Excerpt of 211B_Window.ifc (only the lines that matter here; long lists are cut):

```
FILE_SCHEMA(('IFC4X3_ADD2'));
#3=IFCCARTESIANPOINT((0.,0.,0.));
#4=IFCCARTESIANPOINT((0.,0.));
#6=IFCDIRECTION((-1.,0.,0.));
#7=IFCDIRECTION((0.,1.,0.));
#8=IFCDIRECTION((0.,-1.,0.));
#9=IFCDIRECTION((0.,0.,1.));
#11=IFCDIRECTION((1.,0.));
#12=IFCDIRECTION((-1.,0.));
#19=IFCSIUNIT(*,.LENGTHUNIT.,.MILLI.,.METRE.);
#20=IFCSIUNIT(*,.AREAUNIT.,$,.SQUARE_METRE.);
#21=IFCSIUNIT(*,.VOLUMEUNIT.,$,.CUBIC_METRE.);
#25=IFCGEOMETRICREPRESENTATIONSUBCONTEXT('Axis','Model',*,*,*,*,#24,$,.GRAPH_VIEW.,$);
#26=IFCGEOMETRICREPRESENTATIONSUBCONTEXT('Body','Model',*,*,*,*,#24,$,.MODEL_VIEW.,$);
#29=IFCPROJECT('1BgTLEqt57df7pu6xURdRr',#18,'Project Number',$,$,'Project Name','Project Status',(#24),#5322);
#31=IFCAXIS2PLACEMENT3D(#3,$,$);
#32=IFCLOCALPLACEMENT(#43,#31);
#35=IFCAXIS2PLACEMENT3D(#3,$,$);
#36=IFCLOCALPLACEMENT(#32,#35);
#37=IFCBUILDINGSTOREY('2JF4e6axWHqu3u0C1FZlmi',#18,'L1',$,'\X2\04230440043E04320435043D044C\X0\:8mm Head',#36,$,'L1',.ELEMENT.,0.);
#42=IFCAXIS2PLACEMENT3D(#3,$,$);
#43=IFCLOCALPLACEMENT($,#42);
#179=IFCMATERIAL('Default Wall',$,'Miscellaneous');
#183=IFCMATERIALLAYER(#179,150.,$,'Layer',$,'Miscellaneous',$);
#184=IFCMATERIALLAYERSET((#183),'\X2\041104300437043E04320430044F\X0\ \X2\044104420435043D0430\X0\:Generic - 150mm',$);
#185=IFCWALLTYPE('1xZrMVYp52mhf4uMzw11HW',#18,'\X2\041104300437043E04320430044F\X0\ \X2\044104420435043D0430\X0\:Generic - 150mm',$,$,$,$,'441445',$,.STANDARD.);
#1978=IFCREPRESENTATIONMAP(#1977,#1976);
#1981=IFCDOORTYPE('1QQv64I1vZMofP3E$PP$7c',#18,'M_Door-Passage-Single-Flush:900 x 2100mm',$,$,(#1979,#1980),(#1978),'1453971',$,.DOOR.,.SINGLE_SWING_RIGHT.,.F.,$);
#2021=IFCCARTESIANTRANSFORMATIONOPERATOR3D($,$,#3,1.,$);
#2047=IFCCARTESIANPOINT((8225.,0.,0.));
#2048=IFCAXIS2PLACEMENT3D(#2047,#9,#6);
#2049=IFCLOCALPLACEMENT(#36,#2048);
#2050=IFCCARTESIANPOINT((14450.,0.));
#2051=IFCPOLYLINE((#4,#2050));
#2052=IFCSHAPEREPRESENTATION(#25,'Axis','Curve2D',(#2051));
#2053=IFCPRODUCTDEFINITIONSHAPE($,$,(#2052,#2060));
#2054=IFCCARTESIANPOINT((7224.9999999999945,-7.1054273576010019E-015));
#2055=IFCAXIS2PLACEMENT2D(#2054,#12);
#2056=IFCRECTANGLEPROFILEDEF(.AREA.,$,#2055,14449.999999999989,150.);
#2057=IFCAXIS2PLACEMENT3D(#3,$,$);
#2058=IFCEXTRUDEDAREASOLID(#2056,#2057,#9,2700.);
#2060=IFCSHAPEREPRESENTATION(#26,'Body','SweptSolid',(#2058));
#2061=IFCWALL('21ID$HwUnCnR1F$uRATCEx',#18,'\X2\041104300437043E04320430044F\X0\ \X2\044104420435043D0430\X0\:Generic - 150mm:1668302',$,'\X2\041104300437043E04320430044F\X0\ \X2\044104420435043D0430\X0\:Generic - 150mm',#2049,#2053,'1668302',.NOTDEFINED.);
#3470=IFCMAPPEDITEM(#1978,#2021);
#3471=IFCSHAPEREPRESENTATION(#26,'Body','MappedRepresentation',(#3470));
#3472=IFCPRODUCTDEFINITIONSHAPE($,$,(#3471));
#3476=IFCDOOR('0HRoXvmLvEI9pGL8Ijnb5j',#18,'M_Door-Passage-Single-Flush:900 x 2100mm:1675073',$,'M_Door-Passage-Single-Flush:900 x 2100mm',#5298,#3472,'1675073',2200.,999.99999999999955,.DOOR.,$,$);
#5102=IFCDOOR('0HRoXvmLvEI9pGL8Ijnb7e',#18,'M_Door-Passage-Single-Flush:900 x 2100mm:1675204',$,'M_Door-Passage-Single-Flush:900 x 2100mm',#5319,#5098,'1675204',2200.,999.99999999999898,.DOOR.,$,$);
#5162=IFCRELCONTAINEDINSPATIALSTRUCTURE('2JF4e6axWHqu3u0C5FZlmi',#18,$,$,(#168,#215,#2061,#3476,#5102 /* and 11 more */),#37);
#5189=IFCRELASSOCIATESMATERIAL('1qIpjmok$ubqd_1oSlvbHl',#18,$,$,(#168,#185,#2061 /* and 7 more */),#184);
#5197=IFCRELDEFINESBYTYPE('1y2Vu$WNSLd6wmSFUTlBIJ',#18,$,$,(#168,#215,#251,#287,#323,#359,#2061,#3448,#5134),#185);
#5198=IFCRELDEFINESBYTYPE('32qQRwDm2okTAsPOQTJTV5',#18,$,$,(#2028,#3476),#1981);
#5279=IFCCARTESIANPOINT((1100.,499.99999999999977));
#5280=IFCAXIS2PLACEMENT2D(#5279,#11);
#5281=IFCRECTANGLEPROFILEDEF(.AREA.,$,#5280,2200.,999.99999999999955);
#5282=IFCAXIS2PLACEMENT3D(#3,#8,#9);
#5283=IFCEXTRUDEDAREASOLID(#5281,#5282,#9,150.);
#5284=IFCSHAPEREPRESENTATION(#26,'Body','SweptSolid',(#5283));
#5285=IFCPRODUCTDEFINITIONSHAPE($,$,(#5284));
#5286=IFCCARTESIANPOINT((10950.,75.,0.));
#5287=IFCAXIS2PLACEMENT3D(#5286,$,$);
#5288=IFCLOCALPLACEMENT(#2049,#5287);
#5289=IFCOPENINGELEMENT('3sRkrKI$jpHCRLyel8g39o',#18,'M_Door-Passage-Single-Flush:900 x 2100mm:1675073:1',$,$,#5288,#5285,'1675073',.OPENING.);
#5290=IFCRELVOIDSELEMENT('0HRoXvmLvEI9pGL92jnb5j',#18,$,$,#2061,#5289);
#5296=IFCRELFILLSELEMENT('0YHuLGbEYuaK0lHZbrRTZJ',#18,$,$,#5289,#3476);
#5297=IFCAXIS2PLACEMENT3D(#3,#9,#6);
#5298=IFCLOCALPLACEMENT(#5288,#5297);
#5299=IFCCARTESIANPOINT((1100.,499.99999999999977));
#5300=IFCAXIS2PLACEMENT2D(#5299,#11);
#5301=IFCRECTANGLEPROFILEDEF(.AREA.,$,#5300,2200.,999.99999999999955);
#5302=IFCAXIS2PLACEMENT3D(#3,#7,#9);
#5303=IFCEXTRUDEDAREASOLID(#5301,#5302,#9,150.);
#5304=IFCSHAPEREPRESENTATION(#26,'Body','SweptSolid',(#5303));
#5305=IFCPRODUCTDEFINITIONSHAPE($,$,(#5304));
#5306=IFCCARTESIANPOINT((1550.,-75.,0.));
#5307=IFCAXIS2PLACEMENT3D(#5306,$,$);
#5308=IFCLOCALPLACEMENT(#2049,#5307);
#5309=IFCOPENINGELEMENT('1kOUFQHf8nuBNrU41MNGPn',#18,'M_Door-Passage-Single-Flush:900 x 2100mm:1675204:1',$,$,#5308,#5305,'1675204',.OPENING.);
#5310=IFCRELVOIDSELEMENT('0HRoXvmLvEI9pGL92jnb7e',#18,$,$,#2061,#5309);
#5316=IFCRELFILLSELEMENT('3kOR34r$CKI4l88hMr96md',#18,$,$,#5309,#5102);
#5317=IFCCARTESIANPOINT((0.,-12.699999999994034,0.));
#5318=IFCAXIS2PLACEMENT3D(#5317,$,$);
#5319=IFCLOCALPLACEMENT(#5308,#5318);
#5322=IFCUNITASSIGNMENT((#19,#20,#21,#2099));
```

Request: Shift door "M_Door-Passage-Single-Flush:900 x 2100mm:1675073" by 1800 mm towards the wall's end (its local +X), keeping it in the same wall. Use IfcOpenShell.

```python
import ifcopenshell
import ifcopenshell.api.geometry
import ifcopenshell.util.placement

model = ifcopenshell.open("211B_Window.ifc")

door = model.by_id(3476)
opening = door.FillsVoids[0].RelatingOpeningElement
wall = opening.VoidsElements[0].RelatingBuildingElement

wall_matrix = ifcopenshell.util.placement.get_local_placement(wall.ObjectPlacement)
shift = wall_matrix[:3, 0] * 1800.0
before = ifcopenshell.util.placement.get_local_placement(door.ObjectPlacement)[:3, 3].copy()

# The door is placed relative to its opening, so it follows when the opening moves.
matrix = ifcopenshell.util.placement.get_local_placement(opening.ObjectPlacement)
matrix[:3, 3] += shift
ifcopenshell.api.geometry.edit_object_placement(
    model, product=opening, matrix=matrix, is_si=False, should_transform_children=True
)

after = ifcopenshell.util.placement.get_local_placement(door.ObjectPlacement)[:3, 3]
print("door moved by", (after - before).round(3) + 0.0)

model.write("211B_Window_updated.ifc")
```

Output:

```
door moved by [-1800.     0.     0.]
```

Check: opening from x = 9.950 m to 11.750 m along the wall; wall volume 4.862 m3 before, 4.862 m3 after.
